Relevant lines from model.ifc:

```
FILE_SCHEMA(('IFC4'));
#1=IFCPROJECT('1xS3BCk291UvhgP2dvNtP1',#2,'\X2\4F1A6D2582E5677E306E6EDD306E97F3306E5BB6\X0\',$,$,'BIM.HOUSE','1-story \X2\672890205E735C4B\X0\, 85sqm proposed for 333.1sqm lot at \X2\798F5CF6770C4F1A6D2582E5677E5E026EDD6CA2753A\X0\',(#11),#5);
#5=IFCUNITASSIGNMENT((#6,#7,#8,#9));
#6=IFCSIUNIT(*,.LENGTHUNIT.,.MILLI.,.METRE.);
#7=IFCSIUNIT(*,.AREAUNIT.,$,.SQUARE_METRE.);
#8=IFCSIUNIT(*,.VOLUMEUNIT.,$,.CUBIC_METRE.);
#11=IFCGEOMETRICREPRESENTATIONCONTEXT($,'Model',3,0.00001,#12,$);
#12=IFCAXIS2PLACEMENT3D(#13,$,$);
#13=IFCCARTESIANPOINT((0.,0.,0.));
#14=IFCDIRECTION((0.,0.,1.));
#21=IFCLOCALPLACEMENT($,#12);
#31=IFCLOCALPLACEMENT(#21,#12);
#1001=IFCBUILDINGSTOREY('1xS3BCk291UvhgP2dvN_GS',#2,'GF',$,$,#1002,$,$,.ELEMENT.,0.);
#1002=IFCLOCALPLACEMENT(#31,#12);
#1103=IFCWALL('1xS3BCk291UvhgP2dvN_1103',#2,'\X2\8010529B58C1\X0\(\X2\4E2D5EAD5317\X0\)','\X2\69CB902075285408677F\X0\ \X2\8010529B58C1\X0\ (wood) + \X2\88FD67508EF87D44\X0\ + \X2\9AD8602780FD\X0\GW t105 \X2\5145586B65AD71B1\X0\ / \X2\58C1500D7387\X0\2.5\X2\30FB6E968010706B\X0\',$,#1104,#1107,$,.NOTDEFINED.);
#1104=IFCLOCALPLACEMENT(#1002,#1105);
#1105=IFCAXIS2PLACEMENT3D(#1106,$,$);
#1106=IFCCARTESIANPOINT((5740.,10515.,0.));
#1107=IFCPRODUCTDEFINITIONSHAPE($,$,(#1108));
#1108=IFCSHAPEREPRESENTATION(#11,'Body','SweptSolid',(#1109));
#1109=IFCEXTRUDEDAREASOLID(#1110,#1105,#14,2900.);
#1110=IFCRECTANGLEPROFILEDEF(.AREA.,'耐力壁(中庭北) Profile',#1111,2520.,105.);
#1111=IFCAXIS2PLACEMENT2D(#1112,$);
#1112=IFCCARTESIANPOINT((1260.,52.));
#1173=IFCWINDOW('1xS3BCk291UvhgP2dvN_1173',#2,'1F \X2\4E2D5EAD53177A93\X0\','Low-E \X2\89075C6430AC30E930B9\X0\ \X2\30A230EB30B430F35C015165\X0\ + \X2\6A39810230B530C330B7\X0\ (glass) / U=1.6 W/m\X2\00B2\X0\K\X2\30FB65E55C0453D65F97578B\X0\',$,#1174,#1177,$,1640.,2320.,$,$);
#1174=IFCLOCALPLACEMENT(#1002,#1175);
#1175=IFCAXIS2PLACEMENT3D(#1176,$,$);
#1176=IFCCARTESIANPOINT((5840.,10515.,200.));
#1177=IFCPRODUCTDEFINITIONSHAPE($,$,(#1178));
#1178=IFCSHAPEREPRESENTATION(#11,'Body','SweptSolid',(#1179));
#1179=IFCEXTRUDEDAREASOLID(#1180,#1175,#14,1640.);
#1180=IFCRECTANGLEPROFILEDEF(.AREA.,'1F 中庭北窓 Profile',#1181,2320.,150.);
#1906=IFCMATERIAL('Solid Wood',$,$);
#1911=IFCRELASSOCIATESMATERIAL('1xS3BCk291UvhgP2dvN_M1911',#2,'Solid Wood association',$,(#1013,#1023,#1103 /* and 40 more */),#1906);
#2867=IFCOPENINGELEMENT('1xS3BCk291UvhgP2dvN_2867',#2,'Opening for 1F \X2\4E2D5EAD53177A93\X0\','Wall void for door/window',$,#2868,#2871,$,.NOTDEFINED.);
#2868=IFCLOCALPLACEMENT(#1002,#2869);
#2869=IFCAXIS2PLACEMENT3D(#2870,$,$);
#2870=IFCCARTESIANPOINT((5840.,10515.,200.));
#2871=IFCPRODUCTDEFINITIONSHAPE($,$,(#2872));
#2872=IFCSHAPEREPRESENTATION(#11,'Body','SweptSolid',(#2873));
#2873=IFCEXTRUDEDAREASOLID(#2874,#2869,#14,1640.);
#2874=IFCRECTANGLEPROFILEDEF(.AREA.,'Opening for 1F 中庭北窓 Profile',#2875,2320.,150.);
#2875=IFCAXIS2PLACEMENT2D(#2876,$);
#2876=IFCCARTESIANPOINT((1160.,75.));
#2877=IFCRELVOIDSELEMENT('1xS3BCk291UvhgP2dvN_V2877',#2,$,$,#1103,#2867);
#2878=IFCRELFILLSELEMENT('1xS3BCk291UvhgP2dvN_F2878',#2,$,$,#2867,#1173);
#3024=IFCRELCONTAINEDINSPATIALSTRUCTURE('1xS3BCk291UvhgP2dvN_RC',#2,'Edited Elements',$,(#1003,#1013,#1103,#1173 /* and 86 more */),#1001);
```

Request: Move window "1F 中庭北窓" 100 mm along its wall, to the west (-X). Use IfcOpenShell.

```python
import ifcopenshell
import ifcopenshell.api.geometry
import ifcopenshell.util.placement
import ifcopenshell.util.unit

model = ifcopenshell.open("model.ifc")
unit_scale = ifcopenshell.util.unit.calculate_unit_scale(model)

window = model.by_id(1173)
opening = window.FillsVoids[0].RelatingOpeningElement
wall = opening.VoidsElements[0].RelatingBuildingElement

wall_matrix = ifcopenshell.util.placement.get_local_placement(wall.ObjectPlacement)
shift = wall_matrix[:3, 0] * -0.1 / unit_scale
before = ifcopenshell.util.placement.get_local_placement(window.ObjectPlacement)[:3, 3].copy()

# The window is not placed relative to its opening, so move both.
for product in (opening, window):
    matrix = ifcopenshell.util.placement.get_local_placement(product.ObjectPlacement)
    matrix[:3, 3] += shift
    ifcopenshell.api.geometry.edit_object_placement(model, product=product, matrix=matrix, is_si=False)

after = ifcopenshell.util.placement.get_local_placement(window.ObjectPlacement)[:3, 3]
print("window moved by", (after - before).round(3) + 0.0)

model.write("model_updated.ifc")
```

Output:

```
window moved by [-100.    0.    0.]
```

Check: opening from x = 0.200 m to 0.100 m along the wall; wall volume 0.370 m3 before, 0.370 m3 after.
